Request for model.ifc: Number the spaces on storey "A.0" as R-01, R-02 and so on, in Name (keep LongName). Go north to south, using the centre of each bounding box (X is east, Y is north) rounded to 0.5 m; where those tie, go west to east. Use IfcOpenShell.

First a look at what the model holds.

```python
import ifcopenshell
import ifcopenshell.util.element
import ifcopenshell.util.placement

model = ifcopenshell.open("model.ifc")
print(model.schema)
storey = next(s for s in model.by_type("IfcBuildingStorey") if s.Name == "A.0")
spaces = [e for e in ifcopenshell.util.element.get_decomposition(storey) if e.is_a("IfcSpace")]
for e in sorted(spaces, key=lambda e: e.id()):
    origin = ifcopenshell.util.placement.get_local_placement(e.ObjectPlacement)[:3, 3]
    print(e.id(), e.Name, e.LongName, origin.round(2) + 0.0, sep=" | ")
```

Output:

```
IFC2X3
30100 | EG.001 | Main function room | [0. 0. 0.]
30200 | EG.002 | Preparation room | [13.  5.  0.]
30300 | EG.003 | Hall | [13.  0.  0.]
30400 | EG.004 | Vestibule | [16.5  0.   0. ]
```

```python
import ifcopenshell
import ifcopenshell.geom
import ifcopenshell.util.element
import ifcopenshell.util.shape

model = ifcopenshell.open("model.ifc")
settings = ifcopenshell.geom.settings()
settings.set("use-world-coords", True)


def centre(element):
    shape = ifcopenshell.geom.create_shape(settings, element)
    return ifcopenshell.util.shape.get_bbox_centroid(shape.geometry)


storey = next(s for s in model.by_type("IfcBuildingStorey") if s.Name == "A.0")
spaces = [e for e in ifcopenshell.util.element.get_decomposition(storey) if e.is_a("IfcSpace")]

# Insertion points can sit at a corner or the storey origin, so sort by the geometry (in metres).
centres = {e: centre(e) for e in spaces}
spaces.sort(key=lambda e: (-round(centres[e][1] / 0.5), centres[e][0]))

for i, e in enumerate(spaces, start=1):
    number = f"R-{i:02d}"
    e.Name = number
    print(e.id(), number)

model.write("model_rev.ifc")
```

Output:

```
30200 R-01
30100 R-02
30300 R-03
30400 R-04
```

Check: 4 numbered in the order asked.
